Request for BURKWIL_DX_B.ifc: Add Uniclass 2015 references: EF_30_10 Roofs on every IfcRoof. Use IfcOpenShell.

First a look at what the model holds.

```python
import ifcopenshell

model = ifcopenshell.open("BURKWIL_DX_B.ifc")
print(model.schema)
print("classifications:", [c.Name for c in model.by_type("IfcClassification")])
for ifc_class in ("IfcDoor", "IfcRoof", "IfcStair", "IfcWall", "IfcWindow"):
    print(ifc_class, len(model.by_type(ifc_class)))
```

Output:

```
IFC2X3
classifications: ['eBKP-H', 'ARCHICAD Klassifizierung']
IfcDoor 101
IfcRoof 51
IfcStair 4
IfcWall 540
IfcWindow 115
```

```python
import ifcopenshell
import ifcopenshell.api.classification

model = ifcopenshell.open("BURKWIL_DX_B.ifc")

# IFC2X3 requires Source and Edition and has no link from the project to the system.
system = model.create_entity("IfcClassification", Source="NBS", Edition="2015", Name="Uniclass 2015")

codes = {
    "IfcRoof": ("EF_30_10", "Roofs"),
}
for ifc_class, (code, name) in codes.items():
    products = model.by_type(ifc_class)
    ifcopenshell.api.classification.add_reference(
        model, products=products, classification=system, identification=code, name=name
    )
    print(code, len(products))

model.write("BURKWIL_DX_B_v2.ifc")
```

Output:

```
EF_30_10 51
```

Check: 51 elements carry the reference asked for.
